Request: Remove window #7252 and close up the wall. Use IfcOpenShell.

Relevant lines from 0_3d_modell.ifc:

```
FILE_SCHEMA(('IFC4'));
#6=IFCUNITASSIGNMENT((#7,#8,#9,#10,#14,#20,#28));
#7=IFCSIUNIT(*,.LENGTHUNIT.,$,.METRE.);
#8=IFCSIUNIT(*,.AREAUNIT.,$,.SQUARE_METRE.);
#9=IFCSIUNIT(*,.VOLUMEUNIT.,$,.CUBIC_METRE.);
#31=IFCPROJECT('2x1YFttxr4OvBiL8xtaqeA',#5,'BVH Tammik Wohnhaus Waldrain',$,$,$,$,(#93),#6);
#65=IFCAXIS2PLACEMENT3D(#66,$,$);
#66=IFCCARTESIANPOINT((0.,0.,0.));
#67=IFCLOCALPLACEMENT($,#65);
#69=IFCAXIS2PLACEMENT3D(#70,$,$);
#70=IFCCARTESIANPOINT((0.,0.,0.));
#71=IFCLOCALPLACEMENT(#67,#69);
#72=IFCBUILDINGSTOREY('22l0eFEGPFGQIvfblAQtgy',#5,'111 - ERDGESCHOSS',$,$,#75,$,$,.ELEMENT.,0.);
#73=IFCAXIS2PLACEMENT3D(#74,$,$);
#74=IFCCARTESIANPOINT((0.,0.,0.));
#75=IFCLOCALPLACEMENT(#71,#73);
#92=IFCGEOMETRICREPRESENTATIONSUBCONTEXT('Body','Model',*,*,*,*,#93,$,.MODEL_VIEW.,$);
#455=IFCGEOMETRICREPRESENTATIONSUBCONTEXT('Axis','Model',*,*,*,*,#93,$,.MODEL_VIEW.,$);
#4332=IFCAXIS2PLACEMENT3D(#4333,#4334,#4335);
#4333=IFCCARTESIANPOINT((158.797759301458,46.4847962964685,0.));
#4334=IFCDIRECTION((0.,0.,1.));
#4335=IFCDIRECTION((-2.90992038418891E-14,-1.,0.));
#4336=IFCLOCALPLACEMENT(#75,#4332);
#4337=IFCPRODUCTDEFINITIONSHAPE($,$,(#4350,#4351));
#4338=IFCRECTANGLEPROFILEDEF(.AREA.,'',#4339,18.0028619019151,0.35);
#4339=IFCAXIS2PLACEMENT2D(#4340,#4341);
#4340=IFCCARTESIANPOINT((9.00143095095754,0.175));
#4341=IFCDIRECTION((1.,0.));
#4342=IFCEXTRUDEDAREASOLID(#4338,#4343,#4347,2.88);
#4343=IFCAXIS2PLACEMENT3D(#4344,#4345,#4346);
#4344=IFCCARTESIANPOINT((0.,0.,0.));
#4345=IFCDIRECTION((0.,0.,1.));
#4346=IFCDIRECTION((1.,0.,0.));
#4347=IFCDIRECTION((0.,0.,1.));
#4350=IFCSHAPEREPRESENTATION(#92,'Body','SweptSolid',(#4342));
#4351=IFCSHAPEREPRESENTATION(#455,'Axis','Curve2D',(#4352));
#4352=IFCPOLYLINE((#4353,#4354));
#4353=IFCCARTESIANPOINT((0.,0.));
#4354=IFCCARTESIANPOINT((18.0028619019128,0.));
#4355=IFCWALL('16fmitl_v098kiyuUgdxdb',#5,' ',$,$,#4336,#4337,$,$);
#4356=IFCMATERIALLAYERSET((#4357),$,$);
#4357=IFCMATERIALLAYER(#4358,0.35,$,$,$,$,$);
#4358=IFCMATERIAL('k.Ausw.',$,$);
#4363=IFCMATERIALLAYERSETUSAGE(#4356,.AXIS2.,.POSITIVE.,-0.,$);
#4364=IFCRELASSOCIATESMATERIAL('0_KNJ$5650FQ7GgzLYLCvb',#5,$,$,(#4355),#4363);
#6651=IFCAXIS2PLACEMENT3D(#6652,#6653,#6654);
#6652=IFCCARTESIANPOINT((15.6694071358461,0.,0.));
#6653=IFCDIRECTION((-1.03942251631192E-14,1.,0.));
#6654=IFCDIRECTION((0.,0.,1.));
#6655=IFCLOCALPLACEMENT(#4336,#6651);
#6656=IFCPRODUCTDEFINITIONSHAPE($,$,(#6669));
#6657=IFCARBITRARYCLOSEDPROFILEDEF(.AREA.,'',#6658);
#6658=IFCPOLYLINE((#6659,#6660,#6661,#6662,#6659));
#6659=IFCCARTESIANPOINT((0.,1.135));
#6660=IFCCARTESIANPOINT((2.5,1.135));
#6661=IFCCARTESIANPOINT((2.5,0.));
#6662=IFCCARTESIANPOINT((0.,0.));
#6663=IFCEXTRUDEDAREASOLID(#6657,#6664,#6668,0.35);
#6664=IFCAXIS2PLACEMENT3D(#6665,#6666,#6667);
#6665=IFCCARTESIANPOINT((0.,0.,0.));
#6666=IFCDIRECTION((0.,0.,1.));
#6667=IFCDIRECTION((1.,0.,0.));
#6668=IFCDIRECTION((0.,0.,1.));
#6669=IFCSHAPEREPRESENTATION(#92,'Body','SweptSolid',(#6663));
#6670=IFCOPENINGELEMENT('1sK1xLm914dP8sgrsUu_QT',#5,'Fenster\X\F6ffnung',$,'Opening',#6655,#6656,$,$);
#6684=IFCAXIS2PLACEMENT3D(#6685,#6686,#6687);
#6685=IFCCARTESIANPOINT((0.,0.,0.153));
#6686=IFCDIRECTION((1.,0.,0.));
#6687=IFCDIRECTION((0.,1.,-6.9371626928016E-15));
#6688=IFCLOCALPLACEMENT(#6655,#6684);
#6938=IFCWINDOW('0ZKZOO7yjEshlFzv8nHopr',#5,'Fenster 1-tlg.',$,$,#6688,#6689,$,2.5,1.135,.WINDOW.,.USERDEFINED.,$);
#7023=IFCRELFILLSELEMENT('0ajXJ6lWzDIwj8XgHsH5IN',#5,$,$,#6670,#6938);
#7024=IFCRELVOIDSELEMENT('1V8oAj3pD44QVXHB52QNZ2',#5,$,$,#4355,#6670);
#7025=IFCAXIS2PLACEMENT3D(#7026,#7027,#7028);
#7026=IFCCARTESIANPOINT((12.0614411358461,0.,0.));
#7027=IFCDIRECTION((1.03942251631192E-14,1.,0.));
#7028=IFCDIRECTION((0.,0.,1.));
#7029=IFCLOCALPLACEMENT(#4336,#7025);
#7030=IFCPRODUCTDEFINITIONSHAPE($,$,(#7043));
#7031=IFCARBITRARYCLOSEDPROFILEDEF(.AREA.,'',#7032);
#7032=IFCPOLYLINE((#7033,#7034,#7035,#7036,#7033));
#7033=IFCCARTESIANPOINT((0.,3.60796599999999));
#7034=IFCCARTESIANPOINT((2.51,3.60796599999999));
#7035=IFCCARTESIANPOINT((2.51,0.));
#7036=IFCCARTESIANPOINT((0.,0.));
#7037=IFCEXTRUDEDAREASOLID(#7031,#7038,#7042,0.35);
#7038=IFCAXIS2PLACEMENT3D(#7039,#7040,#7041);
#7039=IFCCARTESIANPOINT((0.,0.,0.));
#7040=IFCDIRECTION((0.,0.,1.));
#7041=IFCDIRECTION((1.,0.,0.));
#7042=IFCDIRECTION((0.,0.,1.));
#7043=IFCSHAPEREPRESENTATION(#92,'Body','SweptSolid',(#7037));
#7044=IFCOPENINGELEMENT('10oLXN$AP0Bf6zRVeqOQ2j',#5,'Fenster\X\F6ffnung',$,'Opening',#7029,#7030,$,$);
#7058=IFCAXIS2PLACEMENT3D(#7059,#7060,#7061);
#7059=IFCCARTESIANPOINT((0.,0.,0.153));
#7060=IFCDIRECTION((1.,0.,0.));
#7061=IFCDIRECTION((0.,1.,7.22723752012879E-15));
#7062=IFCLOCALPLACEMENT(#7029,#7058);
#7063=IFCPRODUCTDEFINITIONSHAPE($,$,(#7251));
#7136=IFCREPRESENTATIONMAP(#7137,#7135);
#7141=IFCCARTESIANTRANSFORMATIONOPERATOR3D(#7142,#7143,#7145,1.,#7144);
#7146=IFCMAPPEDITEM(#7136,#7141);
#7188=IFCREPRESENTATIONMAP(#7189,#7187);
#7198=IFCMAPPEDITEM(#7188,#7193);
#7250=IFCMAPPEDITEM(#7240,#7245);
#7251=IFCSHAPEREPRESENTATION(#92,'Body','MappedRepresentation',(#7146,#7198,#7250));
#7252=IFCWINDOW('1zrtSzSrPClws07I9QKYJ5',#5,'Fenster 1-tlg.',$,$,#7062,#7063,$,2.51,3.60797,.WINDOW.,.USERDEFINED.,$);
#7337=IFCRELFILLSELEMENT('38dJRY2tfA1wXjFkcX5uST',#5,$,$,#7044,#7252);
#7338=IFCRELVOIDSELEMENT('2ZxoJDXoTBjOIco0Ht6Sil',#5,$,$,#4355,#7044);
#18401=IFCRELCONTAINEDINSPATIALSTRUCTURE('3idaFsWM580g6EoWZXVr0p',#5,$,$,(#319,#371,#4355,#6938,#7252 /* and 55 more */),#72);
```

```python
import ifcopenshell
import ifcopenshell.api.feature
import ifcopenshell.api.root
import ifcopenshell.geom
import ifcopenshell.util.shape

model = ifcopenshell.open("0_3d_modell.ifc")
settings = ifcopenshell.geom.settings()


def volume(element):
    """Net volume in cubic metres, openings subtracted."""
    shape = ifcopenshell.geom.create_shape(settings, element)
    return ifcopenshell.util.shape.get_volume(shape.geometry)


window = model.by_guid("1zrtSzSrPClws07I9QKYJ5")
opening = window.FillsVoids[0].RelatingOpeningElement
wall = opening.VoidsElements[0].RelatingBuildingElement
before = volume(wall)

ifcopenshell.api.root.remove_product(model, product=window)
ifcopenshell.api.feature.remove_feature(model, feature=opening)

after = volume(wall)

print(f"wall volume {before:.3f} -> {after:.3f} m3")

model.write("0_3d_modell_edited.ifc")
```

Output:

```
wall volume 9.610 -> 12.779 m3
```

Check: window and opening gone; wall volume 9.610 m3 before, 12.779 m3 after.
